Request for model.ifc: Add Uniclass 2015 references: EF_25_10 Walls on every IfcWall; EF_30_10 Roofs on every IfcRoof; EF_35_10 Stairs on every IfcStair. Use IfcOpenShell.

First a look at what the model holds.

```python
import ifcopenshell

model = ifcopenshell.open("model.ifc")
print(model.schema)
print("classifications:", [c.Name for c in model.by_type("IfcClassification")])
for ifc_class in ("IfcDoor", "IfcRoof", "IfcStair", "IfcWall", "IfcWindow"):
    print(ifc_class, len(model.by_type(ifc_class)))
```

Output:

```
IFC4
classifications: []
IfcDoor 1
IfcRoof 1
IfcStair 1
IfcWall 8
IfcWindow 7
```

```python
import ifcopenshell
import ifcopenshell.api.classification

model = ifcopenshell.open("model.ifc")

system = ifcopenshell.api.classification.add_classification(model, classification="Uniclass 2015")

codes = {
    "IfcWall": ("EF_25_10", "Walls"),
    "IfcRoof": ("EF_30_10", "Roofs"),
    "IfcStair": ("EF_35_10", "Stairs"),
}
for ifc_class, (code, name) in codes.items():
    products = model.by_type(ifc_class)
    ifcopenshell.api.classification.add_reference(
        model, products=products, classification=system, identification=code, name=name
    )
    print(code, len(products))

model.write("model_updated.ifc")
```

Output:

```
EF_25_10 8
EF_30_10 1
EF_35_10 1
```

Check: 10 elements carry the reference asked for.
